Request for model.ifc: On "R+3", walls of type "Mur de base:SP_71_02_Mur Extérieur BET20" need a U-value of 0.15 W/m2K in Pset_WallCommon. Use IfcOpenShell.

First a look at what the model holds.

```python
import ifcopenshell
import ifcopenshell.util.element

model = ifcopenshell.open("model.ifc")
print(model.schema)
storey = next(s for s in model.by_type("IfcBuildingStorey") if s.Name == "R+3")
walls = [e for e in ifcopenshell.util.element.get_decomposition(storey) if e.is_a("IfcWall")]
seen = {}
for e in walls:
    element_type = ifcopenshell.util.element.get_type(e)
    key = (element_type.Name if element_type != e and element_type else None, ifcopenshell.util.element.get_pset(e, "Pset_WallCommon", "ThermalTransmittance"))
    seen[key] = seen.get(key, 0) + 1
for (name, value), count in sorted(seen.items(), key=str):
    print(count, "x", name, "|", value)
```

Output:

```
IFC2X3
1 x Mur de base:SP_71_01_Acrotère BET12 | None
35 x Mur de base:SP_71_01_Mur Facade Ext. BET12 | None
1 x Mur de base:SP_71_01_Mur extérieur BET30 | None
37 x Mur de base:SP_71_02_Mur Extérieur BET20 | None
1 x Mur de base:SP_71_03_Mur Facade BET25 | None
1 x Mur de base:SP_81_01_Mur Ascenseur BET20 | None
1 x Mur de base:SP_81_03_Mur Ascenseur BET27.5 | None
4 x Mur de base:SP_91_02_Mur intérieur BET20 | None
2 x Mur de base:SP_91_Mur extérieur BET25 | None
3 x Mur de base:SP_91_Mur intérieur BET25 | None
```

```python
import ifcopenshell
import ifcopenshell.api.pset
import ifcopenshell.util.element

model = ifcopenshell.open("model.ifc")

storey = next(s for s in model.by_type("IfcBuildingStorey") if s.Name == "R+3")
walls = [e for e in ifcopenshell.util.element.get_decomposition(storey) if e.is_a("IfcWall")]

count = 0
for e in walls:
    element_type = ifcopenshell.util.element.get_type(e)
    if element_type in (None, e) or element_type.Name != "Mur de base:SP_71_02_Mur Extérieur BET20":
        continue
    # add_pset returns the element's existing set when there is one.
    pset = ifcopenshell.api.pset.add_pset(model, product=e, name="Pset_WallCommon")
    ifcopenshell.api.pset.edit_pset(model, pset=pset, properties={"ThermalTransmittance": 0.15})
    count += 1

print(count, "walls updated")

model.write("model_v2.ifc")
```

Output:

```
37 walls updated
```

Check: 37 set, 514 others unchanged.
